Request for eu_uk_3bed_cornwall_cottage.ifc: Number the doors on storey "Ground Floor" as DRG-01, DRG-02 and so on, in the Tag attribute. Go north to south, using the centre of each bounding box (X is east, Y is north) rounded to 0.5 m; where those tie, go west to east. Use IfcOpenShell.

First a look at what the model holds.

```python
import ifcopenshell
import ifcopenshell.util.element
import ifcopenshell.util.placement

model = ifcopenshell.open("eu_uk_3bed_cornwall_cottage.ifc")
print(model.schema)
storey = next(s for s in model.by_type("IfcBuildingStorey") if s.Name == "Ground Floor")
doors = [e for e in ifcopenshell.util.element.get_decomposition(storey) if e.is_a("IfcDoor")]
for e in sorted(doors, key=lambda e: e.id()):
    origin = ifcopenshell.util.placement.get_local_placement(e.ObjectPlacement)[:3, 3]
    print(e.id(), e.Tag, e.Name, origin.round(2) + 0.0, sep=" | ")
```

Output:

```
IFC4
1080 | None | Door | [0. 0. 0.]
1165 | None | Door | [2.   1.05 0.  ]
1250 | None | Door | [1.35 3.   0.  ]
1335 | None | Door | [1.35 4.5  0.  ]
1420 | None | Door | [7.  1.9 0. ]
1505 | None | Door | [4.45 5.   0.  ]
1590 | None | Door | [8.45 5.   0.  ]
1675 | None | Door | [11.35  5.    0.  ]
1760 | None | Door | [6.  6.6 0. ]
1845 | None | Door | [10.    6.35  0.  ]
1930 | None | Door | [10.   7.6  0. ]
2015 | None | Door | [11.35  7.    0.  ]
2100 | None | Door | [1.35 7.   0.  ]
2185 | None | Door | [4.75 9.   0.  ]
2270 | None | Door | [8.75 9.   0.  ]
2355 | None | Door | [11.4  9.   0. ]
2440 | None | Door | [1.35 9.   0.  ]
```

```python
import ifcopenshell
import ifcopenshell.geom
import ifcopenshell.util.element
import ifcopenshell.util.shape

model = ifcopenshell.open("eu_uk_3bed_cornwall_cottage.ifc")
settings = ifcopenshell.geom.settings()
settings.set("use-world-coords", True)


def centre(element):
    shape = ifcopenshell.geom.create_shape(settings, element)
    return ifcopenshell.util.shape.get_bbox_centroid(shape.geometry)


storey = next(s for s in model.by_type("IfcBuildingStorey") if s.Name == "Ground Floor")
doors = [e for e in ifcopenshell.util.element.get_decomposition(storey) if e.is_a("IfcDoor")]

# Insertion points can sit at a corner or the storey origin, so sort by the geometry (in metres).
centres = {e: centre(e) for e in doors}
doors.sort(key=lambda e: (-round(centres[e][1] / 0.5), centres[e][0]))

for i, e in enumerate(doors, start=1):
    number = f"DRG-{i:02d}"
    e.Tag = number
    print(e.id(), number)

model.write("eu_uk_3bed_cornwall_cottage_edited.ifc")
```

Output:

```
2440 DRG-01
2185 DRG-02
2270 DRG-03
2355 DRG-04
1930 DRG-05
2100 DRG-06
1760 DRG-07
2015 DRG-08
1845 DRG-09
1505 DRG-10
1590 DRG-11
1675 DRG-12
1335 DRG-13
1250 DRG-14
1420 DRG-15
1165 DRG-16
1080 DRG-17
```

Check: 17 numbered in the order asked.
